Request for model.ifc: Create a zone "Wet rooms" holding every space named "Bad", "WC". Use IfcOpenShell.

First a look at what the model holds.

```python
import ifcopenshell

model = ifcopenshell.open("model.ifc")
print(model.schema)
seen = {}
for space in model.by_type("IfcSpace"):
    seen[space.LongName] = seen.get(space.LongName, 0) + 1
for name, count in sorted(seen.items(), key=str):
    print(count, "x", name)
print("zones:", [z.Name for z in model.by_type("IfcZone")][:20])
```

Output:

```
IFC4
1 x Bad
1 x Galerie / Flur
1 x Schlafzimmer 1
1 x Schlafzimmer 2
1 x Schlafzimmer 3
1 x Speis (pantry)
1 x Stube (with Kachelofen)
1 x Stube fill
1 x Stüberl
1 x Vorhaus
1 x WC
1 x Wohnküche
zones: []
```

```python
import ifcopenshell
import ifcopenshell.api.group
import ifcopenshell.api.root

model = ifcopenshell.open("model.ifc")

names = {"Bad", "WC"}
spaces = [s for s in model.by_type("IfcSpace") if s.LongName in names]

zone = ifcopenshell.api.root.create_entity(model, ifc_class="IfcZone", name="Wet rooms")
ifcopenshell.api.group.assign_group(model, products=spaces, group=zone)
print(len(spaces), "spaces in", zone.Name)

model.write("model-out.ifc")
```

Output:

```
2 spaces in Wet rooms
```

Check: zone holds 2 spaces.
